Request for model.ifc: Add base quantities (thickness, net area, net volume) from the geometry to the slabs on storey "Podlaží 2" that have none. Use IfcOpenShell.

First a look at what the model holds.

```python
import ifcopenshell
import ifcopenshell.util.element
import ifcopenshell.util.unit

model = ifcopenshell.open("model.ifc")
print(model.schema)
for unit_type in ("LENGTHUNIT", "AREAUNIT", "VOLUMEUNIT"):
    print(unit_type, ifcopenshell.util.unit.calculate_unit_scale(model, unit_type))
storey = next(s for s in model.by_type("IfcBuildingStorey") if s.Name == "Podlaží 2")
slabs = [e for e in ifcopenshell.util.element.get_decomposition(storey) if e.is_a("IfcSlab")]
for e in sorted(slabs, key=lambda e: e.id()):
    print(e.id(), e.is_a(), e.Name, list(ifcopenshell.util.element.get_psets(e, qtos_only=True)), sep=" | ")
```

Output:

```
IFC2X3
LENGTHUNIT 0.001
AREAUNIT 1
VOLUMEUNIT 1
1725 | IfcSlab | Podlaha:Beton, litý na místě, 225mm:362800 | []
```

```python
import ifcopenshell
import ifcopenshell.api.pset
import ifcopenshell.geom
import ifcopenshell.util.element
import ifcopenshell.util.shape
import ifcopenshell.util.unit

model = ifcopenshell.open("model.ifc")
unit_scale = ifcopenshell.util.unit.calculate_unit_scale(model)
area_scale = ifcopenshell.util.unit.calculate_unit_scale(model, "AREAUNIT")
volume_scale = ifcopenshell.util.unit.calculate_unit_scale(model, "VOLUMEUNIT")
settings = ifcopenshell.geom.settings()

storey = next(s for s in model.by_type("IfcBuildingStorey") if s.Name == "Podlaží 2")
slabs = [e for e in ifcopenshell.util.element.get_decomposition(storey) if e.is_a("IfcSlab")]

for e in sorted(slabs, key=lambda e: e.id()):
    if ifcopenshell.util.element.get_psets(e, qtos_only=True, should_inherit=False):
        continue
    # Geometry comes back in metres, in the element's own axes.
    shape = ifcopenshell.geom.create_shape(settings, e)
    values = {
        "Width": ifcopenshell.util.shape.get_z(shape.geometry) / unit_scale,
        "NetArea": ifcopenshell.util.shape.get_footprint_area(shape.geometry) / area_scale,
        "NetVolume": ifcopenshell.util.shape.get_volume(shape.geometry) / volume_scale,
    }
    qto = ifcopenshell.api.pset.add_qto(model, product=e, name="BaseQuantities")
    ifcopenshell.api.pset.edit_qto(model, qto=qto, properties=values)
    print(e.id(), {k: round(v, 3) for k, v in values.items()})

model.write("model_v2.ifc")
```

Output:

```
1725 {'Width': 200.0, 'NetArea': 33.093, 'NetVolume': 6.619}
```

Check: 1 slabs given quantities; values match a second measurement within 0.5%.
